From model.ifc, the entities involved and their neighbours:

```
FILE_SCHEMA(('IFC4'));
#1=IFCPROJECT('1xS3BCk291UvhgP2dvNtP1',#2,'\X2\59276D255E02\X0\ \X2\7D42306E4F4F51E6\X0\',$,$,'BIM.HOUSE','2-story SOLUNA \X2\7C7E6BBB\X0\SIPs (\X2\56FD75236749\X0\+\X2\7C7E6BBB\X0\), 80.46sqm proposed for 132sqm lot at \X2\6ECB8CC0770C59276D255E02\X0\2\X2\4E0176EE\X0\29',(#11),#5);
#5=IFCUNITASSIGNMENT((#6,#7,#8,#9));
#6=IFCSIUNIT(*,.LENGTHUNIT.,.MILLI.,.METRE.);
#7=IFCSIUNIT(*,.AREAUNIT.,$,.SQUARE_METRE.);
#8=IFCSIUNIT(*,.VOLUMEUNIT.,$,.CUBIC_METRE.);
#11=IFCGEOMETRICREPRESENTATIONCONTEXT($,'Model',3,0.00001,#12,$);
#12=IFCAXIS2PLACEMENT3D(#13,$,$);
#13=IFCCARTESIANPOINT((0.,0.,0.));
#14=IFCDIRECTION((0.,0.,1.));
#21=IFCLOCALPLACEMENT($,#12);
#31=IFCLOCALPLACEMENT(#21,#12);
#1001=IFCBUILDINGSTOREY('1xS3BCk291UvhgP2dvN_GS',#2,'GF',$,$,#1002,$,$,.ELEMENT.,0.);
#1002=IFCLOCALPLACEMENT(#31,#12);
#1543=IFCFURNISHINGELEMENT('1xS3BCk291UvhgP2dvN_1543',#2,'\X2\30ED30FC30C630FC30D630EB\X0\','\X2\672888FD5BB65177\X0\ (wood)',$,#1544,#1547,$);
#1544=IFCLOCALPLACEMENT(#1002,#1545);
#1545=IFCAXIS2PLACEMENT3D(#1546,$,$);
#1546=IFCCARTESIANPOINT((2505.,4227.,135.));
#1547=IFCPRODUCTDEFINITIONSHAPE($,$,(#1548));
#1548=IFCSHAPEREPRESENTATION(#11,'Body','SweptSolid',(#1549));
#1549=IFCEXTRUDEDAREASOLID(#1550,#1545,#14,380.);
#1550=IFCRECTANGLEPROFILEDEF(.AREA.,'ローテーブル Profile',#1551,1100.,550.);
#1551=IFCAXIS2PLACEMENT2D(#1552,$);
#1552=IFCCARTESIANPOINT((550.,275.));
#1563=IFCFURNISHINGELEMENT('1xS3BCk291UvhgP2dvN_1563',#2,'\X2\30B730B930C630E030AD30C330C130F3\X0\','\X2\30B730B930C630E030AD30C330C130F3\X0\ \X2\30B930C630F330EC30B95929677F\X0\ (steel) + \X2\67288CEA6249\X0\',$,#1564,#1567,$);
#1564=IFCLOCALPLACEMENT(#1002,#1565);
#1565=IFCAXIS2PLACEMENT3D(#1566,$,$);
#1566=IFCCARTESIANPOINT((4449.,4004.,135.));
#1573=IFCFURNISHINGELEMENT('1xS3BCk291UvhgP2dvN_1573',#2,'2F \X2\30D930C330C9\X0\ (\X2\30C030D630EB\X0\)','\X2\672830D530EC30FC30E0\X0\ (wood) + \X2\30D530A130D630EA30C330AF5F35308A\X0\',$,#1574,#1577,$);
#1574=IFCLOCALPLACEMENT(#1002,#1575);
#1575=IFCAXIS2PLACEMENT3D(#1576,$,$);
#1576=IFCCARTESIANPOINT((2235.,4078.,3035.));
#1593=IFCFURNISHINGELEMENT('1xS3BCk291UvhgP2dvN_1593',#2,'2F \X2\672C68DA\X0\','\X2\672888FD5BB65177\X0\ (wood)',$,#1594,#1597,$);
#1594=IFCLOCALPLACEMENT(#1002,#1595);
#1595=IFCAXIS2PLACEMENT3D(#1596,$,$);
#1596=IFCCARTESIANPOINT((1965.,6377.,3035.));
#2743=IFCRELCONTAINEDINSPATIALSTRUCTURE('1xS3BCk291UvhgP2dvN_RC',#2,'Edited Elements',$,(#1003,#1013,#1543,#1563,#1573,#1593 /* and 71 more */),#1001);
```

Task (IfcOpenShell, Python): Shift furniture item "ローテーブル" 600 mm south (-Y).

```python
import ifcopenshell
import ifcopenshell.api.geometry
import ifcopenshell.util.placement
import ifcopenshell.util.unit

model = ifcopenshell.open("model.ifc")
unit_scale = ifcopenshell.util.unit.calculate_unit_scale(model)

item = model.by_guid("1xS3BCk291UvhgP2dvN_1543")
matrix = ifcopenshell.util.placement.get_local_placement(item.ObjectPlacement)
matrix[1, 3] -= 0.6 / unit_scale
ifcopenshell.api.geometry.edit_object_placement(model, product=item, matrix=matrix, is_si=False)

print(ifcopenshell.util.placement.get_local_placement(item.ObjectPlacement).round(3) + 0.0)

model.write("model_updated.ifc")
```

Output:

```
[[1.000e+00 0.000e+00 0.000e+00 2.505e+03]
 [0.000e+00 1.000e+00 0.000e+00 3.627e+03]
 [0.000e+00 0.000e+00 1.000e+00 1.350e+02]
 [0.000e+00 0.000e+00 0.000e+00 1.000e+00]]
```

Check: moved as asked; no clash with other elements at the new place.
